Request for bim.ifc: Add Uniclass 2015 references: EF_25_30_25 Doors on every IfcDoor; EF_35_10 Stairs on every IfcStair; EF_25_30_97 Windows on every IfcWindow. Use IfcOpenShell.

First a look at what the model holds.

```python
import ifcopenshell

model = ifcopenshell.open("bim.ifc")
print(model.schema)
print("classifications:", [c.Name for c in model.by_type("IfcClassification")])
for ifc_class in ("IfcDoor", "IfcRoof", "IfcStair", "IfcWall", "IfcWindow"):
    print(ifc_class, len(model.by_type(ifc_class)))
```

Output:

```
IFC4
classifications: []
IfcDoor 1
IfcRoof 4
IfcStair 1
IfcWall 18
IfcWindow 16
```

```python
import ifcopenshell
import ifcopenshell.api.classification

model = ifcopenshell.open("bim.ifc")

system = ifcopenshell.api.classification.add_classification(model, classification="Uniclass 2015")

codes = {
    "IfcDoor": ("EF_25_30_25", "Doors"),
    "IfcStair": ("EF_35_10", "Stairs"),
    "IfcWindow": ("EF_25_30_97", "Windows"),
}
for ifc_class, (code, name) in codes.items():
    products = model.by_type(ifc_class)
    ifcopenshell.api.classification.add_reference(
        model, products=products, classification=system, identification=code, name=name
    )
    print(code, len(products))

model.write("bim_rev.ifc")
```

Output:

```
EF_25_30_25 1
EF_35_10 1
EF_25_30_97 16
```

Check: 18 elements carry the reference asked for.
